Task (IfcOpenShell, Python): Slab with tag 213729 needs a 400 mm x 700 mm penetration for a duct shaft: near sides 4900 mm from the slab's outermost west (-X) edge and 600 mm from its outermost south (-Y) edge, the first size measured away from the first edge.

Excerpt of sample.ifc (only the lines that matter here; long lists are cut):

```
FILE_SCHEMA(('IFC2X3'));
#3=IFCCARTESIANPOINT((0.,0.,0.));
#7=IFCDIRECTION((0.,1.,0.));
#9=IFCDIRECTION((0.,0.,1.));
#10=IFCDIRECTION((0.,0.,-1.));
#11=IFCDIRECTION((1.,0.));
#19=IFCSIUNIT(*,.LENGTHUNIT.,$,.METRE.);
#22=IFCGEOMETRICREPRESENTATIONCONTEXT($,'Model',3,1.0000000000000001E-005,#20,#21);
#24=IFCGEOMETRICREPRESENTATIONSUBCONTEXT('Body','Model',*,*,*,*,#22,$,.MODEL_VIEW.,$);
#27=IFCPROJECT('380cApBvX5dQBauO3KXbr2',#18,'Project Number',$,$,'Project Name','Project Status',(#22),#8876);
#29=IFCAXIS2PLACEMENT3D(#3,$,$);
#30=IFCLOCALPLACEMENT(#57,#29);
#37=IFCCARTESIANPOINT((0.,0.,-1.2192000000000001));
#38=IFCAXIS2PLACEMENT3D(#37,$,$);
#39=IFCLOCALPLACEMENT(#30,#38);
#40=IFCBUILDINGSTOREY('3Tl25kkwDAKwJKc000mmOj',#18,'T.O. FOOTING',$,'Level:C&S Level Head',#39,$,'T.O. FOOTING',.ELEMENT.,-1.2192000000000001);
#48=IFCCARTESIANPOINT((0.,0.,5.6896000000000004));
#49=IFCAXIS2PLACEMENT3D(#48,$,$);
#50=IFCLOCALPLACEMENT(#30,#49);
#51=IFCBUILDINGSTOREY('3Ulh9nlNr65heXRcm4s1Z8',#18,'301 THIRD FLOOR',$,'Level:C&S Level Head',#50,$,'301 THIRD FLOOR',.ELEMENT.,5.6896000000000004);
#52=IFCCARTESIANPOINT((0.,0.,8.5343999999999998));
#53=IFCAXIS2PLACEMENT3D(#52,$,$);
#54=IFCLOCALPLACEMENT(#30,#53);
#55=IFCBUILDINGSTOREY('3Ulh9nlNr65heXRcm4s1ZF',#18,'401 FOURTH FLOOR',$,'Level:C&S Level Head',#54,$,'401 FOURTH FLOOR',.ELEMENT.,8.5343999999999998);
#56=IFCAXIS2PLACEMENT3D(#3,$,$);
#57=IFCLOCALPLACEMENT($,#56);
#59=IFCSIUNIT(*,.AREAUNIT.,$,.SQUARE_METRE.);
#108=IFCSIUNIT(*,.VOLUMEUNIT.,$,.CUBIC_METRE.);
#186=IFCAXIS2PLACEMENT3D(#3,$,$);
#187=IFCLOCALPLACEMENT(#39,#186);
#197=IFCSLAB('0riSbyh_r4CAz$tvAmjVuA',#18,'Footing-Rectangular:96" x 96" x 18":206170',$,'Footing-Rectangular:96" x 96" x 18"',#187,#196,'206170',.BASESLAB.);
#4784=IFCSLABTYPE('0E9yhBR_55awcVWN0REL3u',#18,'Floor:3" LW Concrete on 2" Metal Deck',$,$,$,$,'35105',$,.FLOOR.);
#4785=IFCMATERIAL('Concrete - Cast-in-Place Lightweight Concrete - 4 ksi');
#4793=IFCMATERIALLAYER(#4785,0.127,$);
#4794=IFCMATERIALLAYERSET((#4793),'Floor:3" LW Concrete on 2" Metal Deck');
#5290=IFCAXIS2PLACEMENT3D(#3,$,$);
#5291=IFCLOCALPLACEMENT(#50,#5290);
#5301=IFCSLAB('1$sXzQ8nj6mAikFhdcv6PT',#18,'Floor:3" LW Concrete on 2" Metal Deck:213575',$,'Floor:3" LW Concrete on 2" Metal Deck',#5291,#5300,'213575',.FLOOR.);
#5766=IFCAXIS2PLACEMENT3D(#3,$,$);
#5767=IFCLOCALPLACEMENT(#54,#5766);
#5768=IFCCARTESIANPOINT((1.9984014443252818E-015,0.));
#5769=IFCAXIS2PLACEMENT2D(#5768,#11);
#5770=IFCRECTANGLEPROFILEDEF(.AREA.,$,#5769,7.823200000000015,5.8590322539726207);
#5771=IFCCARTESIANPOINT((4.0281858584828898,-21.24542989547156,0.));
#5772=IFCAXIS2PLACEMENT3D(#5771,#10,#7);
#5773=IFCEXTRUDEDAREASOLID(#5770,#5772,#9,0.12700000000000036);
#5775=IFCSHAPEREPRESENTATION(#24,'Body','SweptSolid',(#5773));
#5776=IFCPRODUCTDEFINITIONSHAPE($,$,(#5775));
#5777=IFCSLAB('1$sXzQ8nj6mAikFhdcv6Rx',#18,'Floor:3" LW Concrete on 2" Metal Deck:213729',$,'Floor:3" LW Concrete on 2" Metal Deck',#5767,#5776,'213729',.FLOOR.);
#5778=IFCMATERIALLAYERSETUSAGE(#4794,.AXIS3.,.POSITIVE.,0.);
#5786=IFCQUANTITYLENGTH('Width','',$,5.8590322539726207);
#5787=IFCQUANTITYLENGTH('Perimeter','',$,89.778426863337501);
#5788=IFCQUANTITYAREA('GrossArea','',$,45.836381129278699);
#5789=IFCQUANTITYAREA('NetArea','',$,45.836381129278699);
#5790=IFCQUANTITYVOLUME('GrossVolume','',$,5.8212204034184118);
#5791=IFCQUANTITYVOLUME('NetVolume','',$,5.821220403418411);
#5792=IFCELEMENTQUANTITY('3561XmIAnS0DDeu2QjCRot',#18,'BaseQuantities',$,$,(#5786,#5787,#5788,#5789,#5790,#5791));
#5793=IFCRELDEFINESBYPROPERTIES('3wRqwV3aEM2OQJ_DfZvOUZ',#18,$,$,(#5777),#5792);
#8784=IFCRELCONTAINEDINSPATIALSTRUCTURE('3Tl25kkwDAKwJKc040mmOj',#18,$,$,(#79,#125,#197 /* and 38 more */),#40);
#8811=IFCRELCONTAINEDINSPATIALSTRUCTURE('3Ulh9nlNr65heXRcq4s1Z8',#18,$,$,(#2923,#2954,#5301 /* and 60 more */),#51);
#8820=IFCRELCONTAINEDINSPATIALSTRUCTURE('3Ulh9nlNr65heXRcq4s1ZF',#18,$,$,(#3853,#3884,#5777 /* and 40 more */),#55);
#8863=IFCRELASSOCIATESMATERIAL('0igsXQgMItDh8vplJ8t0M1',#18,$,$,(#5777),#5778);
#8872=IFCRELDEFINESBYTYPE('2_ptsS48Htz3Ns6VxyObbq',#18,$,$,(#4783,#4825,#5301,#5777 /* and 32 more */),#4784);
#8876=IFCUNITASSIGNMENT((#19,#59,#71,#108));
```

```python
import numpy as np
import ifcopenshell
import ifcopenshell.api.feature
import ifcopenshell.api.geometry
import ifcopenshell.api.pset
import ifcopenshell.api.root
import ifcopenshell.geom
import ifcopenshell.util.element
import ifcopenshell.util.placement
import ifcopenshell.util.representation
import ifcopenshell.util.shape
import ifcopenshell.util.unit

model = ifcopenshell.open("sample.ifc")
unit_scale = ifcopenshell.util.unit.calculate_unit_scale(model)
area_scale = ifcopenshell.util.unit.calculate_unit_scale(model, "AREAUNIT")
volume_scale = ifcopenshell.util.unit.calculate_unit_scale(model, "VOLUMEUNIT")
settings = ifcopenshell.geom.settings()


def volume(element):
    """Net volume in cubic metres, openings subtracted."""
    shape = ifcopenshell.geom.create_shape(settings, element)
    return ifcopenshell.util.shape.get_volume(shape.geometry)


slab = model.by_guid("1$sXzQ8nj6mAikFhdcv6Rx")
before = volume(slab)

# Extent in the slab's own axes, in metres. The edges named are its -X and -Y sides.
slab_shape = ifcopenshell.geom.create_shape(settings, slab)
vertices = ifcopenshell.util.shape.get_vertices(slab_shape.geometry)
x_min, y_min, bottom = vertices.min(axis=0)
top = vertices[:, 2].max()

opening = ifcopenshell.api.root.create_entity(model, ifc_class="IfcOpeningElement", name="Duct shaft opening")
context = ifcopenshell.util.representation.get_context(model, "Model", "Body", "MODEL_VIEW")
width, depth = 0.4, 0.7
outline = [(0.0, 0.0), (width, 0.0), (width, depth), (0.0, depth), (0.0, 0.0)]
# Overshoot both faces by 50 mm so the cut is clean.
shape = ifcopenshell.api.geometry.add_slab_representation(
    model, context=context, depth=top - bottom + 0.1, polyline=outline
)
ifcopenshell.api.geometry.assign_representation(model, product=opening, representation=shape)

matrix = ifcopenshell.util.placement.get_local_placement(slab.ObjectPlacement)
matrix[:, 3] = matrix @ np.append(np.array([x_min + 4.9, y_min + 0.6, bottom - 0.05]) / unit_scale, 1.0)
ifcopenshell.api.geometry.edit_object_placement(model, product=opening, matrix=matrix, is_si=False)
ifcopenshell.api.feature.add_feature(model, feature=opening, element=slab)

after = volume(slab)

# Update the slab's stored quantities.
qto = model.by_id(ifcopenshell.util.element.get_pset(slab, "BaseQuantities", should_inherit=False)["id"])
ifcopenshell.api.pset.edit_qto(model, qto=qto, properties={
    "NetArea": after / (top - bottom) / area_scale,
    "NetVolume": after / volume_scale,
})

print(f"slab volume {before:.3f} -> {after:.3f} m3")

model.write("sample_v2.ifc")
```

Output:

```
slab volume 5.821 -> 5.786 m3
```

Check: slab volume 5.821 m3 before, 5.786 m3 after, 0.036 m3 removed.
